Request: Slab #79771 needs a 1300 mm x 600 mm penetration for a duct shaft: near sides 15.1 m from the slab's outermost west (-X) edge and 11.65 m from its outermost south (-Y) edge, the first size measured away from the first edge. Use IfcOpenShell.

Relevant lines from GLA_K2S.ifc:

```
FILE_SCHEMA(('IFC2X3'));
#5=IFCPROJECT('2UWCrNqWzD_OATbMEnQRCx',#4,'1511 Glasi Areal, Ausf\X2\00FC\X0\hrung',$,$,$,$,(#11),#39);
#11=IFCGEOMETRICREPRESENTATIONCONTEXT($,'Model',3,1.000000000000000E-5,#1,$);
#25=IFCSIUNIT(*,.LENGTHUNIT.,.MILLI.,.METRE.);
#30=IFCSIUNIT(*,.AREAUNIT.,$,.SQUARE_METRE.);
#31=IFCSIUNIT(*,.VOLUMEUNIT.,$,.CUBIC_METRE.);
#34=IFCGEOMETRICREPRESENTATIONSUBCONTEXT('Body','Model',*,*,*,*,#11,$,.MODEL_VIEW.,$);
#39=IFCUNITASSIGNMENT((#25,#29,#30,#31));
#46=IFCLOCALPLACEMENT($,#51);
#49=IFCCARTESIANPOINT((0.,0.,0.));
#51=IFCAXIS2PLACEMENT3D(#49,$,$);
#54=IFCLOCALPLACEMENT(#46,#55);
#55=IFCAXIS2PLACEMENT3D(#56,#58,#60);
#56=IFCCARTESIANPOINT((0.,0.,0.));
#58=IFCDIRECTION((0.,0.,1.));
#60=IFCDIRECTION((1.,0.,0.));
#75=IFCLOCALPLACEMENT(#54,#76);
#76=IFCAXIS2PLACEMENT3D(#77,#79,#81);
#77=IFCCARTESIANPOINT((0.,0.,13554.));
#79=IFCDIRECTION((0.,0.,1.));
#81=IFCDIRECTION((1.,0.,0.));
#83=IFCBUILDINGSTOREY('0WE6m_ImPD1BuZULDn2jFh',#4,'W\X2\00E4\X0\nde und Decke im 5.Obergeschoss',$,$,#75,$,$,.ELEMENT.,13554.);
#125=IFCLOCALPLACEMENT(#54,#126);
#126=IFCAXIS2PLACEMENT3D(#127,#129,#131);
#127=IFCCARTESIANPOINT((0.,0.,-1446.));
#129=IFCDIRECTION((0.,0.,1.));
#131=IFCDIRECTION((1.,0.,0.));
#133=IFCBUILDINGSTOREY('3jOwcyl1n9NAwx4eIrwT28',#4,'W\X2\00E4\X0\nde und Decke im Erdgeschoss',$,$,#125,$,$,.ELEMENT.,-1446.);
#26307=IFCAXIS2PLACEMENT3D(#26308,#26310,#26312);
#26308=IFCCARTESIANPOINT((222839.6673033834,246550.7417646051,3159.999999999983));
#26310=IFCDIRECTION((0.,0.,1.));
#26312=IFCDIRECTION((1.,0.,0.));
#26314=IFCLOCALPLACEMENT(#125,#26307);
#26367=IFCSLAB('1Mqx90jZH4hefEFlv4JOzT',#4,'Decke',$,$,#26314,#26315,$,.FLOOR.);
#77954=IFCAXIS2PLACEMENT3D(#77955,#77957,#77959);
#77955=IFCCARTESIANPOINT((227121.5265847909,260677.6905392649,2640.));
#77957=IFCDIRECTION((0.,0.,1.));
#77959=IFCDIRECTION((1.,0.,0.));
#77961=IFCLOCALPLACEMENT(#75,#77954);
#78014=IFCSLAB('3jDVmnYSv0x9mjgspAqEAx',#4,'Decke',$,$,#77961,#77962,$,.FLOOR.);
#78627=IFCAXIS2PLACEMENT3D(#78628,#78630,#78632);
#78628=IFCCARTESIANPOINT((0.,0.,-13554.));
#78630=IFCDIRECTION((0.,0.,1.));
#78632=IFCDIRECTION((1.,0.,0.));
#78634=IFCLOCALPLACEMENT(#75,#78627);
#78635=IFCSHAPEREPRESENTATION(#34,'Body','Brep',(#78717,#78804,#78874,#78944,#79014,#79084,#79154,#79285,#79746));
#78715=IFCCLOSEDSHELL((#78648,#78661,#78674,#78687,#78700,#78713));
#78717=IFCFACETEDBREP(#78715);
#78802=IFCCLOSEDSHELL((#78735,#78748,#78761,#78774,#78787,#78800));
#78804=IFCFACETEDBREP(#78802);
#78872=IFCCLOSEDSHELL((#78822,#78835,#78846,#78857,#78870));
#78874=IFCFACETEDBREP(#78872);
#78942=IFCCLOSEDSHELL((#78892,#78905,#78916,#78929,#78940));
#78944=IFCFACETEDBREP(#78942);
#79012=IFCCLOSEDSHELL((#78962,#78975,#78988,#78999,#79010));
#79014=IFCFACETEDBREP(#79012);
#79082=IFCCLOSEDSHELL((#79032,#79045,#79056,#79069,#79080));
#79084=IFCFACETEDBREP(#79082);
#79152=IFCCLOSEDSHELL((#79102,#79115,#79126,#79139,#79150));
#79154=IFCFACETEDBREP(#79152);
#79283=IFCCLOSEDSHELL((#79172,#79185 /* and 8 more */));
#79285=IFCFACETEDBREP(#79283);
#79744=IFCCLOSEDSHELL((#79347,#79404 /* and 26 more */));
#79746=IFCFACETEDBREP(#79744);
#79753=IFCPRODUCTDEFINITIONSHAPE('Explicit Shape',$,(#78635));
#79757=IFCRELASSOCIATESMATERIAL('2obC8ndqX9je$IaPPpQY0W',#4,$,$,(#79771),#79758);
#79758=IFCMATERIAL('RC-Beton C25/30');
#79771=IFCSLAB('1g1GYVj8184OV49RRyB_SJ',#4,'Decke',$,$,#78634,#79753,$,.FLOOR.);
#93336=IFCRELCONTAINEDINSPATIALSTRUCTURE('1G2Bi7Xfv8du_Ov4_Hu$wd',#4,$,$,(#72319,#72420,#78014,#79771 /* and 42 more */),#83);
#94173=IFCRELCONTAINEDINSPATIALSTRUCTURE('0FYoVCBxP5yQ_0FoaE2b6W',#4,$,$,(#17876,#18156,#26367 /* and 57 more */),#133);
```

```python
import numpy as np
import ifcopenshell
import ifcopenshell.api.feature
import ifcopenshell.api.geometry
import ifcopenshell.api.root
import ifcopenshell.geom
import ifcopenshell.util.placement
import ifcopenshell.util.representation
import ifcopenshell.util.shape
import ifcopenshell.util.unit

model = ifcopenshell.open("GLA_K2S.ifc")
unit_scale = ifcopenshell.util.unit.calculate_unit_scale(model)
settings = ifcopenshell.geom.settings()


def volume(element):
    """Net volume in cubic metres, openings subtracted."""
    shape = ifcopenshell.geom.create_shape(settings, element)
    return ifcopenshell.util.shape.get_volume(shape.geometry)


slab = model.by_id(79771)
before = volume(slab)

# Extent in the slab's own axes, in metres. The edges named are its -X and -Y sides.
slab_shape = ifcopenshell.geom.create_shape(settings, slab)
vertices = ifcopenshell.util.shape.get_vertices(slab_shape.geometry)
x_min, y_min, bottom = vertices.min(axis=0)
top = vertices[:, 2].max()

opening = ifcopenshell.api.root.create_entity(model, ifc_class="IfcOpeningElement", name="Duct shaft opening")
context = ifcopenshell.util.representation.get_context(model, "Model", "Body", "MODEL_VIEW")
width, depth = 1.3, 0.6
outline = [(0.0, 0.0), (width, 0.0), (width, depth), (0.0, depth), (0.0, 0.0)]
# Overshoot both faces by 50 mm so the cut is clean.
shape = ifcopenshell.api.geometry.add_slab_representation(
    model, context=context, depth=top - bottom + 0.1, polyline=outline
)
ifcopenshell.api.geometry.assign_representation(model, product=opening, representation=shape)

matrix = ifcopenshell.util.placement.get_local_placement(slab.ObjectPlacement)
matrix[:, 3] = matrix @ np.append(np.array([x_min + 15.1, y_min + 11.65, bottom - 0.05]) / unit_scale, 1.0)
ifcopenshell.api.geometry.edit_object_placement(model, product=opening, matrix=matrix, is_si=False)
ifcopenshell.api.feature.add_feature(model, feature=opening, element=slab)

after = volume(slab)

print(f"slab volume {before:.3f} -> {after:.3f} m3")

model.write("GLA_K2S_rev.ifc")
```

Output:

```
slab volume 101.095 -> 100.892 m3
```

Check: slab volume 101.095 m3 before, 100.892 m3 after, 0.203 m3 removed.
